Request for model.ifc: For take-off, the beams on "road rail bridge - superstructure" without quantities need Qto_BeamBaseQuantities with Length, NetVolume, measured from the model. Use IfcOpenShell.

First a look at what the model holds.

```python
import ifcopenshell
import ifcopenshell.util.element
import ifcopenshell.util.unit

model = ifcopenshell.open("model.ifc")
print(model.schema)
for unit_type in ("LENGTHUNIT", "AREAUNIT", "VOLUMEUNIT"):
    print(unit_type, ifcopenshell.util.unit.calculate_unit_scale(model, unit_type))
storey = next(s for s in model.by_type("IfcBuildingStorey") if s.Name == "road rail bridge - superstructure")
beams = [e for e in ifcopenshell.util.element.get_decomposition(storey) if e.is_a("IfcBeam")]
for e in sorted(beams, key=lambda e: e.id()):
    print(e.id(), e.is_a(), e.Name, list(ifcopenshell.util.element.get_psets(e, qtos_only=True)), sep=" | ")
```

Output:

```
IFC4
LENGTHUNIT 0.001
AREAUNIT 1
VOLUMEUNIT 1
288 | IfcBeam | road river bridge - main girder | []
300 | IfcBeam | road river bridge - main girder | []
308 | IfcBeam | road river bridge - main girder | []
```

```python
import ifcopenshell
import ifcopenshell.api.pset
import ifcopenshell.geom
import ifcopenshell.util.element
import ifcopenshell.util.shape
import ifcopenshell.util.unit

model = ifcopenshell.open("model.ifc")
unit_scale = ifcopenshell.util.unit.calculate_unit_scale(model)
volume_scale = ifcopenshell.util.unit.calculate_unit_scale(model, "VOLUMEUNIT")
settings = ifcopenshell.geom.settings()

storey = next(s for s in model.by_type("IfcBuildingStorey") if s.Name == "road rail bridge - superstructure")
beams = [e for e in ifcopenshell.util.element.get_decomposition(storey) if e.is_a("IfcBeam")]

for e in sorted(beams, key=lambda e: e.id()):
    if ifcopenshell.util.element.get_psets(e, qtos_only=True, should_inherit=False):
        continue
    # Geometry comes back in metres, in the element's own axes.
    shape = ifcopenshell.geom.create_shape(settings, e)
    values = {
        "Length": ifcopenshell.util.shape.get_max_xyz(shape.geometry) / unit_scale,
        "NetVolume": ifcopenshell.util.shape.get_volume(shape.geometry) / volume_scale,
    }
    qto = ifcopenshell.api.pset.add_qto(model, product=e, name="Qto_BeamBaseQuantities")
    ifcopenshell.api.pset.edit_qto(model, qto=qto, properties=values)
    print(e.id(), {k: round(v, 3) for k, v in values.items()})

model.write("model-out.ifc")
```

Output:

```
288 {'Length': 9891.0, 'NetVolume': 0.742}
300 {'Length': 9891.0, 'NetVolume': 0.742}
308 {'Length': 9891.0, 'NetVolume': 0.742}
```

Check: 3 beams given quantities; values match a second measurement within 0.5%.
